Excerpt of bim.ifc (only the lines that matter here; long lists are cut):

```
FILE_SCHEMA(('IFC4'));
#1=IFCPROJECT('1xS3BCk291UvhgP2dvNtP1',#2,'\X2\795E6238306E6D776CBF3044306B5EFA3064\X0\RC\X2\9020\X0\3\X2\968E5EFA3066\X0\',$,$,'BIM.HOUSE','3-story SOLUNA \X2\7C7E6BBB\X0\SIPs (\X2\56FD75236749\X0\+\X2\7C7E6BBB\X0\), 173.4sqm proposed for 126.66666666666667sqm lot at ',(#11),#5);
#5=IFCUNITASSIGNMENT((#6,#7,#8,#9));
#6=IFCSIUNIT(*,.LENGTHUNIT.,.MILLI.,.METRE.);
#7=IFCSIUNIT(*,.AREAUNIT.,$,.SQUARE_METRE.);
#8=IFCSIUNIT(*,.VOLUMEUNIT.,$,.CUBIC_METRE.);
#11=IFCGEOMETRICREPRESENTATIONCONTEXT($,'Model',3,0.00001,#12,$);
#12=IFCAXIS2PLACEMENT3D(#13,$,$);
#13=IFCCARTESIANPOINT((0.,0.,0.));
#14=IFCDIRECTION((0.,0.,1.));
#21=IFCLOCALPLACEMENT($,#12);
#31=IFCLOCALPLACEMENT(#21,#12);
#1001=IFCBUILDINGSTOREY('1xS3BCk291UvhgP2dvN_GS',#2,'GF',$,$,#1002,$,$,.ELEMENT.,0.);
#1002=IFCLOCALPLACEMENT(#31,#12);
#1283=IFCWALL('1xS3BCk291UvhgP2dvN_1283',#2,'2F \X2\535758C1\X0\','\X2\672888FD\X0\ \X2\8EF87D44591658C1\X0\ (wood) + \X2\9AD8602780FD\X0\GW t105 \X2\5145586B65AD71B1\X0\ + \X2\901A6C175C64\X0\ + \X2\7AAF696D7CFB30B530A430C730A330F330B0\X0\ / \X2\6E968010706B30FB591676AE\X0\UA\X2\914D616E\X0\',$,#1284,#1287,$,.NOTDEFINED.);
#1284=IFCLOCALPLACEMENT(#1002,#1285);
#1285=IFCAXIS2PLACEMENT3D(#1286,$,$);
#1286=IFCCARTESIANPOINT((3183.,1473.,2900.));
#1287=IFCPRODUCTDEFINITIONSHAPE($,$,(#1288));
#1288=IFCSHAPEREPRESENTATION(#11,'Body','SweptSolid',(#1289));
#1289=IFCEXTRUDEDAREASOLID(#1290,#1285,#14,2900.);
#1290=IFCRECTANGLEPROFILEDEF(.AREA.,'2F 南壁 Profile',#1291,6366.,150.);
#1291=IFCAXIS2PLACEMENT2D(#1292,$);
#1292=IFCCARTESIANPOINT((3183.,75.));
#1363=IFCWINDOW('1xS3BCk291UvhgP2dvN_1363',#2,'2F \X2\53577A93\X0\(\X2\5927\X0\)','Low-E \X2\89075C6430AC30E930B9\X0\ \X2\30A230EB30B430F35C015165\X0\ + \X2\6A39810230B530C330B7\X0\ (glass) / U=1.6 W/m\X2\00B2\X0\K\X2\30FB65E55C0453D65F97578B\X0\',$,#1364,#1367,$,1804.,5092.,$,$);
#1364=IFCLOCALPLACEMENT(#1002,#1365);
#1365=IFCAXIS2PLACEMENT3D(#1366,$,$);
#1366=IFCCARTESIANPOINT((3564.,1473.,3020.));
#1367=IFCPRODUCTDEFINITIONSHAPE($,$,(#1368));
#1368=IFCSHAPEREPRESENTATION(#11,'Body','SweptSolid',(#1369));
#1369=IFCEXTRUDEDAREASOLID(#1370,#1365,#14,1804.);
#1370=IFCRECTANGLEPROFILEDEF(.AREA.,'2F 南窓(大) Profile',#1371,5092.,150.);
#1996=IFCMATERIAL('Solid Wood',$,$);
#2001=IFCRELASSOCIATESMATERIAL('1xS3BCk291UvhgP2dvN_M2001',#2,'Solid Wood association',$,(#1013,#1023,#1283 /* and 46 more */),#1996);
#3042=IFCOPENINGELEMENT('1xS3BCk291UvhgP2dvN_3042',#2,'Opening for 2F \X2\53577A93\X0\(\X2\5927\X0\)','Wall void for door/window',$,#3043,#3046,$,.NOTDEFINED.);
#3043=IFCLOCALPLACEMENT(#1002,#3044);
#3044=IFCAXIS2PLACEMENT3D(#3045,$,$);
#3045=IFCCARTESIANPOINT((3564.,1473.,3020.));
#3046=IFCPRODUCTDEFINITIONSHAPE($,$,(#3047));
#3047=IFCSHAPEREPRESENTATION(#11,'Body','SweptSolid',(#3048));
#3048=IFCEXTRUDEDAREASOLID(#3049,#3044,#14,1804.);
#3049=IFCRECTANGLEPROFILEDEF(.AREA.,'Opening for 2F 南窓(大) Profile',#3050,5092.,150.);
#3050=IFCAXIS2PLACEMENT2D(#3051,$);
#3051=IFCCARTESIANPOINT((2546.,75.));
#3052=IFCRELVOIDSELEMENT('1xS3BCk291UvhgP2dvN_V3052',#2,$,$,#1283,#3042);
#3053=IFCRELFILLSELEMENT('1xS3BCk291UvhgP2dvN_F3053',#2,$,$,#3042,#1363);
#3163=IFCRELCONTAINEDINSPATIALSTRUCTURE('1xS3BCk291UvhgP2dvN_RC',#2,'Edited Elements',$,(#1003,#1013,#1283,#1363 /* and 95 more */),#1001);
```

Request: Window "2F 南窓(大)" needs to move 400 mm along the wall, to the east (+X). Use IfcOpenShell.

```python
import ifcopenshell
import ifcopenshell.api.geometry
import ifcopenshell.util.placement
import ifcopenshell.util.unit

model = ifcopenshell.open("bim.ifc")
unit_scale = ifcopenshell.util.unit.calculate_unit_scale(model)

window = model.by_guid("1xS3BCk291UvhgP2dvN_1363")
opening = window.FillsVoids[0].RelatingOpeningElement
wall = opening.VoidsElements[0].RelatingBuildingElement

wall_matrix = ifcopenshell.util.placement.get_local_placement(wall.ObjectPlacement)
shift = wall_matrix[:3, 0] * 0.4 / unit_scale
before = ifcopenshell.util.placement.get_local_placement(window.ObjectPlacement)[:3, 3].copy()

# The window is not placed relative to its opening, so move both.
for product in (opening, window):
    matrix = ifcopenshell.util.placement.get_local_placement(product.ObjectPlacement)
    matrix[:3, 3] += shift
    ifcopenshell.api.geometry.edit_object_placement(model, product=product, matrix=matrix, is_si=False)

after = ifcopenshell.util.placement.get_local_placement(window.ObjectPlacement)[:3, 3]
print("window moved by", (after - before).round(3) + 0.0)

model.write("bim_updated.ifc")
```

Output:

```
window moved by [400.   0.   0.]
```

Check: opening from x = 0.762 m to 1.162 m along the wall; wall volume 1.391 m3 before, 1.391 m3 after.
